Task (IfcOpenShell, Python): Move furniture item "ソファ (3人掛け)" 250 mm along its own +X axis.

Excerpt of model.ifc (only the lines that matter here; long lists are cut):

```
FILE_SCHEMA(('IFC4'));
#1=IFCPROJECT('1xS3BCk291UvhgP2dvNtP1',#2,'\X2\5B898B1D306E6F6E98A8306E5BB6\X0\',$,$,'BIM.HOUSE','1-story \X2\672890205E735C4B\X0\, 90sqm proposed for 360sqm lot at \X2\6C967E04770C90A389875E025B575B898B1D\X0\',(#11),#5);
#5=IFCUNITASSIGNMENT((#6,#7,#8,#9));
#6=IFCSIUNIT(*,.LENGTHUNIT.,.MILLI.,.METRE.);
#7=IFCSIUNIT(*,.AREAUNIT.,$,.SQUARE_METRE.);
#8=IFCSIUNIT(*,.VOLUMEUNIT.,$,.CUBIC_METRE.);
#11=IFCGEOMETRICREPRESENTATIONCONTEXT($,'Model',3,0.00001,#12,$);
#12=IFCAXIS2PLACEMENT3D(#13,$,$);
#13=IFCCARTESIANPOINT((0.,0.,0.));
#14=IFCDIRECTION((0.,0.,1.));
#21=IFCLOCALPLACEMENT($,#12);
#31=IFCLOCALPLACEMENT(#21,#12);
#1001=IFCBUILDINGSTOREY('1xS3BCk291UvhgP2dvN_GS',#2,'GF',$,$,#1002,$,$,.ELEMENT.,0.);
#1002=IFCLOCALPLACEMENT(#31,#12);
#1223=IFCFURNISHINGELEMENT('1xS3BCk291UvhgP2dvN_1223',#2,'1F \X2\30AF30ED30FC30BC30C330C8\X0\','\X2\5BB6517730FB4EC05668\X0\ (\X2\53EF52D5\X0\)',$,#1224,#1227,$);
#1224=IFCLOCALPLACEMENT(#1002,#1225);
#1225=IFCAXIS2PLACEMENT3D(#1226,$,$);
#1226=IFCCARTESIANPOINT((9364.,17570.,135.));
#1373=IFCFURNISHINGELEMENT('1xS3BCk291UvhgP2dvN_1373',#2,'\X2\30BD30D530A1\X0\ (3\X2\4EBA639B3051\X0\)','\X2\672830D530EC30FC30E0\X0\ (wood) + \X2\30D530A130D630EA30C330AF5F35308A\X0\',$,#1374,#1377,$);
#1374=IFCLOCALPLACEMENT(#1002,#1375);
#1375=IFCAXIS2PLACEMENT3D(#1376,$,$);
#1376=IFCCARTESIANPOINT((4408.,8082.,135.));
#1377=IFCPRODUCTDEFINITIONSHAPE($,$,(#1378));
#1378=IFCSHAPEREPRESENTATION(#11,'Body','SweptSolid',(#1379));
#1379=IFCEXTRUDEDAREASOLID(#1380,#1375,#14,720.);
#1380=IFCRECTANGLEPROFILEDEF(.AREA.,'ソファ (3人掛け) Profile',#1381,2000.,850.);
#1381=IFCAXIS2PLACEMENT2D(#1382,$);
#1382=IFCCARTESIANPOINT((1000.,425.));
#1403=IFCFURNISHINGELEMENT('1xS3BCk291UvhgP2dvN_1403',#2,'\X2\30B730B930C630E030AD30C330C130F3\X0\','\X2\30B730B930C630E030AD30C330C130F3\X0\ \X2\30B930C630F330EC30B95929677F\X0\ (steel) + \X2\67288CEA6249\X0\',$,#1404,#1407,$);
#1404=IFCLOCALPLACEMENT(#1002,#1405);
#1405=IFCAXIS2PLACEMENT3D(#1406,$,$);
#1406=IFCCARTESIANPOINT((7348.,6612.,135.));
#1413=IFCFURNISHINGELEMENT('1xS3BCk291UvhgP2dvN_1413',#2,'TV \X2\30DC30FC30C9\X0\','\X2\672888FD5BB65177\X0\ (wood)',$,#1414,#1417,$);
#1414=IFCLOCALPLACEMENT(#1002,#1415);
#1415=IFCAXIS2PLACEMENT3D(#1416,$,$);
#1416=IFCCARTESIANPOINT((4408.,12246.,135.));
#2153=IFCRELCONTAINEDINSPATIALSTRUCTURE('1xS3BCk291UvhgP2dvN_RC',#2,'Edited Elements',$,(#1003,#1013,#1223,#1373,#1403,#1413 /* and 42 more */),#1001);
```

```python
import ifcopenshell
import ifcopenshell.api.geometry
import ifcopenshell.util.placement
import ifcopenshell.util.unit

model = ifcopenshell.open("model.ifc")
unit_scale = ifcopenshell.util.unit.calculate_unit_scale(model)

item = model.by_guid("1xS3BCk291UvhgP2dvN_1373")
matrix = ifcopenshell.util.placement.get_local_placement(item.ObjectPlacement)
matrix[:3, 3] += matrix[:3, 0] * 0.25 / unit_scale
ifcopenshell.api.geometry.edit_object_placement(model, product=item, matrix=matrix, is_si=False)

print(ifcopenshell.util.placement.get_local_placement(item.ObjectPlacement).round(3) + 0.0)

model.write("model_v2.ifc")
```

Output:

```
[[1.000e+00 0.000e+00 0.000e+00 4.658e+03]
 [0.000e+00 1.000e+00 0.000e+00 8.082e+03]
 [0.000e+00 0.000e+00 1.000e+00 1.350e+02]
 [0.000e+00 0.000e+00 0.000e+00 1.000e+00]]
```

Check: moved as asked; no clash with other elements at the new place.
